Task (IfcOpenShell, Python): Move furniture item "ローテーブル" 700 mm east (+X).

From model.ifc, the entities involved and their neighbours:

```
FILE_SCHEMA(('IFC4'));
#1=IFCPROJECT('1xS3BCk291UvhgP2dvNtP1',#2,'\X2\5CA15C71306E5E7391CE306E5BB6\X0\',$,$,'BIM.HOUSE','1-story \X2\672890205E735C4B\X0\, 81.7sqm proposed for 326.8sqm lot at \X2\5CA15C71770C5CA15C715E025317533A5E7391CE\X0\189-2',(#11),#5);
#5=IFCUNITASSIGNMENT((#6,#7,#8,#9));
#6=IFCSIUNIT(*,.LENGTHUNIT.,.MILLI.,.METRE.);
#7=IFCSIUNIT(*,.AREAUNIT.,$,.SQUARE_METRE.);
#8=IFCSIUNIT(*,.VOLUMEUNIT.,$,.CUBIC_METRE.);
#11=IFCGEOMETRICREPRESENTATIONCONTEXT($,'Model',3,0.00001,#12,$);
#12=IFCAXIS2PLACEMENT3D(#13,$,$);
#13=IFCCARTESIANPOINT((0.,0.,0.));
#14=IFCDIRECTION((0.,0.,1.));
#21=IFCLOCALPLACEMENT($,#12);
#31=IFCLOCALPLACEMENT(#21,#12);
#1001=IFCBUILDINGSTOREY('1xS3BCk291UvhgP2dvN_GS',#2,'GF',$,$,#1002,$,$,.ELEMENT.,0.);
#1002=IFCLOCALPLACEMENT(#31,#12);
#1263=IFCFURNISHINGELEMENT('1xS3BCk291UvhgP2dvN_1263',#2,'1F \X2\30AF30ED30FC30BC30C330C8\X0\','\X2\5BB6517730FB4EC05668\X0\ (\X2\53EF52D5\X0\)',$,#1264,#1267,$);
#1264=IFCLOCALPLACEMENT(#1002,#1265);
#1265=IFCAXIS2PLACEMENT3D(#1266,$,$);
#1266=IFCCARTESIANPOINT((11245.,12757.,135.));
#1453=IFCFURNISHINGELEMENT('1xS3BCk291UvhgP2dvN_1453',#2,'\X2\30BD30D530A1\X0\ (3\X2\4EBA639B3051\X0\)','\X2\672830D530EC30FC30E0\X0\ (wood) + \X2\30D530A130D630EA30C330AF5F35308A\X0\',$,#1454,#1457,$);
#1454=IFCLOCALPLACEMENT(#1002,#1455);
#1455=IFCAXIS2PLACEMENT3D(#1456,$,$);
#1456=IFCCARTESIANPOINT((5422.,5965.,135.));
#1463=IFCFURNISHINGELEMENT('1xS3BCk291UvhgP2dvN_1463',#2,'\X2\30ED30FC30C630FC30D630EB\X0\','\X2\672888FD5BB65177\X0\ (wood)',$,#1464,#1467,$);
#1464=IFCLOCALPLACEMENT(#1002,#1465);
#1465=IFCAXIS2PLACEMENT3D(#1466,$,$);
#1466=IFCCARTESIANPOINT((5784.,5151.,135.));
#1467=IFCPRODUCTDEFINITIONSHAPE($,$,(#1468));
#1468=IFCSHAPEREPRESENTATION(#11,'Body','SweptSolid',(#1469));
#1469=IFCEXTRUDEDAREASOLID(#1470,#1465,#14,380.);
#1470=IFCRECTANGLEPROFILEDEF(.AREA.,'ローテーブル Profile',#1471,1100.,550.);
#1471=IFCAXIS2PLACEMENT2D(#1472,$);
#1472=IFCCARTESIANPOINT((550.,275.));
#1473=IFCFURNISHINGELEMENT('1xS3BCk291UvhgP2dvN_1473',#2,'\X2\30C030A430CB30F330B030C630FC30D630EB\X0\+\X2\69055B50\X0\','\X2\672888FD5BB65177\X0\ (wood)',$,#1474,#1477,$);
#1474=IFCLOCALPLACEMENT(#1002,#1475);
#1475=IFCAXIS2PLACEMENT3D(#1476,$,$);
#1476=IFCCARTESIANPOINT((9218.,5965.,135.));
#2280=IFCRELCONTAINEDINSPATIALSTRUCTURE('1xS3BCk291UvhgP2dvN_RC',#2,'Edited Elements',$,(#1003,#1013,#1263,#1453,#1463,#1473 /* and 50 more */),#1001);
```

```python
import ifcopenshell
import ifcopenshell.api.geometry
import ifcopenshell.util.placement

model = ifcopenshell.open("model.ifc")

item = model.by_guid("1xS3BCk291UvhgP2dvN_1463")
matrix = ifcopenshell.util.placement.get_local_placement(item.ObjectPlacement)
matrix[0, 3] += 700.0
ifcopenshell.api.geometry.edit_object_placement(model, product=item, matrix=matrix, is_si=False)

print(ifcopenshell.util.placement.get_local_placement(item.ObjectPlacement).round(3) + 0.0)

model.write("model_updated.ifc")
```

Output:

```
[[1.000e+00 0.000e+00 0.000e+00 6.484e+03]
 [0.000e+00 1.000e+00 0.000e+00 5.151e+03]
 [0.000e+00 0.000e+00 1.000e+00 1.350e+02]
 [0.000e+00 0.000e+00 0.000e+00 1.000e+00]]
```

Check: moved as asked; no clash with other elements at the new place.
